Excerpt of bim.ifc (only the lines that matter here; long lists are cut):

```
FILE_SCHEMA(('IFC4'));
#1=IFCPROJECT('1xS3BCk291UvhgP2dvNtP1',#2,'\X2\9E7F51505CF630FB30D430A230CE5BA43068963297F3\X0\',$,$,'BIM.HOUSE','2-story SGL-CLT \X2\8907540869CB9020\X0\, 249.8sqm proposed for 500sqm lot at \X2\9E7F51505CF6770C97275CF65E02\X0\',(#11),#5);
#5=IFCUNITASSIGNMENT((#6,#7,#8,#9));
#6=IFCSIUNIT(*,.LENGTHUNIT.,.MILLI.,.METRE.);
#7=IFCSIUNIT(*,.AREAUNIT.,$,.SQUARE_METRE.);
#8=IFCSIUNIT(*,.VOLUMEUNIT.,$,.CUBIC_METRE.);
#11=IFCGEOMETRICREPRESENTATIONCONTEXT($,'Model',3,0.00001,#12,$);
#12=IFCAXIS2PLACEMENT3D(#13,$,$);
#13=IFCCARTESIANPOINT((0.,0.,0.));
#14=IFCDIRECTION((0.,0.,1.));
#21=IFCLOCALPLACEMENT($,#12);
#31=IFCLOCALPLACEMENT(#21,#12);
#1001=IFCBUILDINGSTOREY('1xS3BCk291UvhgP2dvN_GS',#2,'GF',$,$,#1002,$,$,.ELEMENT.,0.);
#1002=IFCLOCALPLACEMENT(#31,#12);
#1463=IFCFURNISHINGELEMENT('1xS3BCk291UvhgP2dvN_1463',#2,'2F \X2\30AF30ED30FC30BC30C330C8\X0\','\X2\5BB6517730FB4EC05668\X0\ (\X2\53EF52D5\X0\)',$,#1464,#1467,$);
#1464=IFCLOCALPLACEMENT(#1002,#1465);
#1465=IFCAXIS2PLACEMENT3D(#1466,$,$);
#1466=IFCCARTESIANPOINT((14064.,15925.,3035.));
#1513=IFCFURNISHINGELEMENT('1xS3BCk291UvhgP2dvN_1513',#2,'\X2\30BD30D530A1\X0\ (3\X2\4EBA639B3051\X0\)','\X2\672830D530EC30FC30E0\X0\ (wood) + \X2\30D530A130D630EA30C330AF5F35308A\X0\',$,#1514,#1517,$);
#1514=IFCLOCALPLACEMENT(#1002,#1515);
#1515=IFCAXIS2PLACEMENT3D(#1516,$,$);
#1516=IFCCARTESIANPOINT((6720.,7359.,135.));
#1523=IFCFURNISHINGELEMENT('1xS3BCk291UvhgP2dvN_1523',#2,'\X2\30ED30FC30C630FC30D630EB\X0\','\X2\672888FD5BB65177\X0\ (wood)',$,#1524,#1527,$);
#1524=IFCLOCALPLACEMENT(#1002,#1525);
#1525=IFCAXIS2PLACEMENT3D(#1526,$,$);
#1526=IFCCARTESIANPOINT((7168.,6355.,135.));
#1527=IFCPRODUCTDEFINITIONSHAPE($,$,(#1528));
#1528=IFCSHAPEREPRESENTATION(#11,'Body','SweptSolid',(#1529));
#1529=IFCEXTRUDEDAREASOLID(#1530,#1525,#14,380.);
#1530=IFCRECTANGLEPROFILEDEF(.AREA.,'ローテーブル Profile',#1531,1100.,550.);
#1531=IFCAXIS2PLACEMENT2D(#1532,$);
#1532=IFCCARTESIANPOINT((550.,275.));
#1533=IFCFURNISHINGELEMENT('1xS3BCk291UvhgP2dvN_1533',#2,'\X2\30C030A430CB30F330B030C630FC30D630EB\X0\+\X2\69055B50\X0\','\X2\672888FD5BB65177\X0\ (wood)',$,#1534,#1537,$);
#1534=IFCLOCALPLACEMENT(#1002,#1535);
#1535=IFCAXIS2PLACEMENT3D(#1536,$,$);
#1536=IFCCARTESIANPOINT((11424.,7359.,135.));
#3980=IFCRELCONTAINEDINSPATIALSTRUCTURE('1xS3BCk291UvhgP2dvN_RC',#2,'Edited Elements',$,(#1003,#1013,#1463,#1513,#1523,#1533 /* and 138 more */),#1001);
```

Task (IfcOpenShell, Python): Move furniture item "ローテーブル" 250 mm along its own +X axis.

```python
import ifcopenshell
import ifcopenshell.api.geometry
import ifcopenshell.util.placement
import ifcopenshell.util.unit

model = ifcopenshell.open("bim.ifc")
unit_scale = ifcopenshell.util.unit.calculate_unit_scale(model)

item = model.by_id(1523)
matrix = ifcopenshell.util.placement.get_local_placement(item.ObjectPlacement)
matrix[:3, 3] += matrix[:3, 0] * 0.25 / unit_scale
ifcopenshell.api.geometry.edit_object_placement(model, product=item, matrix=matrix, is_si=False)

print(ifcopenshell.util.placement.get_local_placement(item.ObjectPlacement).round(3) + 0.0)

model.write("bim_rev.ifc")
```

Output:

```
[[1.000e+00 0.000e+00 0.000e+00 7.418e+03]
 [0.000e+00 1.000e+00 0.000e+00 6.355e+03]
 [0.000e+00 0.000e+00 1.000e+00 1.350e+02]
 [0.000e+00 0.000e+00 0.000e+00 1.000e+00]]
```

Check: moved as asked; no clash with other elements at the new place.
